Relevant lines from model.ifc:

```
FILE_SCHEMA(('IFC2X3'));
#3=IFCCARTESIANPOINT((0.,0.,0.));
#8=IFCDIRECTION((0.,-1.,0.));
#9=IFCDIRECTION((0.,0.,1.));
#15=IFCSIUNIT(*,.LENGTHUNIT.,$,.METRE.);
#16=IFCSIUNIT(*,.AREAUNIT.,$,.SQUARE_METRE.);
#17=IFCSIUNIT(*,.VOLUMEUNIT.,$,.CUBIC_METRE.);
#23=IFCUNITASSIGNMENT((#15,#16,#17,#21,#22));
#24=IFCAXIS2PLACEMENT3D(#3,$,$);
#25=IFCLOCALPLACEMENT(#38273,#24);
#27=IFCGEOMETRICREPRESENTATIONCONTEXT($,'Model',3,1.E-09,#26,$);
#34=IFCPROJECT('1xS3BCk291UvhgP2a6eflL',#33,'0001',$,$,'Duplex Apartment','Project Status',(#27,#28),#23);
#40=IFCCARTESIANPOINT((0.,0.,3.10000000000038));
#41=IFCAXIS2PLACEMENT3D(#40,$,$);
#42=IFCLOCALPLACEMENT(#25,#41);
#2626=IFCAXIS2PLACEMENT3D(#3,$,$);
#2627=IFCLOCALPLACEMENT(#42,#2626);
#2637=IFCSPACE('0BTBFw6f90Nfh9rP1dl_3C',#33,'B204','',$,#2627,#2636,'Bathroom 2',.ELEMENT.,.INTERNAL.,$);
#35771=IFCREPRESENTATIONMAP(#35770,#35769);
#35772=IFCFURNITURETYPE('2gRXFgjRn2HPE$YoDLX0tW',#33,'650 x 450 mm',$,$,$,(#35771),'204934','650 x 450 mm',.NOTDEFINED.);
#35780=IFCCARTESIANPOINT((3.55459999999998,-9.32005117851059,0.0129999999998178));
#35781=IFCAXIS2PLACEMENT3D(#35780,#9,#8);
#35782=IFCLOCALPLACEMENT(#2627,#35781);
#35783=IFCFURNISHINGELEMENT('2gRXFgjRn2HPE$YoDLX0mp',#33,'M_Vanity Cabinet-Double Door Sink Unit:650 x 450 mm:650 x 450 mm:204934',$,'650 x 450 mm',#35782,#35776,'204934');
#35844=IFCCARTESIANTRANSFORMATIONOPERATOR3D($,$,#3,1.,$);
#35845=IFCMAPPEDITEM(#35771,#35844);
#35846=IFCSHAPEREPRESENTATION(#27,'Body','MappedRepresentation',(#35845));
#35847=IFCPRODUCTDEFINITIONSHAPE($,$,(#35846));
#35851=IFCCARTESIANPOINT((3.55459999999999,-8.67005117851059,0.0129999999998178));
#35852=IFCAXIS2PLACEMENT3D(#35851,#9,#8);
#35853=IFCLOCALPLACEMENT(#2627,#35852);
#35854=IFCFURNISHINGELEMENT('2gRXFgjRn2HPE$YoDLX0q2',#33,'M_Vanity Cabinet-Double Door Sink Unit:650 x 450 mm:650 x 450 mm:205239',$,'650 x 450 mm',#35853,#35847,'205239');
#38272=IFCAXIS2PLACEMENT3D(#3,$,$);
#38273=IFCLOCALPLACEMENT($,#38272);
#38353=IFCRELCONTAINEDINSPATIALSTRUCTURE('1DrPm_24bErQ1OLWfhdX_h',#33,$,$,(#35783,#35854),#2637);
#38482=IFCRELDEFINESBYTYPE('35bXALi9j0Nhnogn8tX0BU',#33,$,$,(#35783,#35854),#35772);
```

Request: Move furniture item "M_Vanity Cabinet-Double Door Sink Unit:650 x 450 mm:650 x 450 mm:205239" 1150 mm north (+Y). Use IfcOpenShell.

```python
import ifcopenshell
import ifcopenshell.api.geometry
import ifcopenshell.util.placement
import ifcopenshell.util.unit

model = ifcopenshell.open("model.ifc")
unit_scale = ifcopenshell.util.unit.calculate_unit_scale(model)

item = model.by_guid("2gRXFgjRn2HPE$YoDLX0q2")
matrix = ifcopenshell.util.placement.get_local_placement(item.ObjectPlacement)
matrix[1, 3] += 1.15 / unit_scale
ifcopenshell.api.geometry.edit_object_placement(model, product=item, matrix=matrix, is_si=False)

print(ifcopenshell.util.placement.get_local_placement(item.ObjectPlacement).round(3) + 0.0)

model.write("model_v2.ifc")
```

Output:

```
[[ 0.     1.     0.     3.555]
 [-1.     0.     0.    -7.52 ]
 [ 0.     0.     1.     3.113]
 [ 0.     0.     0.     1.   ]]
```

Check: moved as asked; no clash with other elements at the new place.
